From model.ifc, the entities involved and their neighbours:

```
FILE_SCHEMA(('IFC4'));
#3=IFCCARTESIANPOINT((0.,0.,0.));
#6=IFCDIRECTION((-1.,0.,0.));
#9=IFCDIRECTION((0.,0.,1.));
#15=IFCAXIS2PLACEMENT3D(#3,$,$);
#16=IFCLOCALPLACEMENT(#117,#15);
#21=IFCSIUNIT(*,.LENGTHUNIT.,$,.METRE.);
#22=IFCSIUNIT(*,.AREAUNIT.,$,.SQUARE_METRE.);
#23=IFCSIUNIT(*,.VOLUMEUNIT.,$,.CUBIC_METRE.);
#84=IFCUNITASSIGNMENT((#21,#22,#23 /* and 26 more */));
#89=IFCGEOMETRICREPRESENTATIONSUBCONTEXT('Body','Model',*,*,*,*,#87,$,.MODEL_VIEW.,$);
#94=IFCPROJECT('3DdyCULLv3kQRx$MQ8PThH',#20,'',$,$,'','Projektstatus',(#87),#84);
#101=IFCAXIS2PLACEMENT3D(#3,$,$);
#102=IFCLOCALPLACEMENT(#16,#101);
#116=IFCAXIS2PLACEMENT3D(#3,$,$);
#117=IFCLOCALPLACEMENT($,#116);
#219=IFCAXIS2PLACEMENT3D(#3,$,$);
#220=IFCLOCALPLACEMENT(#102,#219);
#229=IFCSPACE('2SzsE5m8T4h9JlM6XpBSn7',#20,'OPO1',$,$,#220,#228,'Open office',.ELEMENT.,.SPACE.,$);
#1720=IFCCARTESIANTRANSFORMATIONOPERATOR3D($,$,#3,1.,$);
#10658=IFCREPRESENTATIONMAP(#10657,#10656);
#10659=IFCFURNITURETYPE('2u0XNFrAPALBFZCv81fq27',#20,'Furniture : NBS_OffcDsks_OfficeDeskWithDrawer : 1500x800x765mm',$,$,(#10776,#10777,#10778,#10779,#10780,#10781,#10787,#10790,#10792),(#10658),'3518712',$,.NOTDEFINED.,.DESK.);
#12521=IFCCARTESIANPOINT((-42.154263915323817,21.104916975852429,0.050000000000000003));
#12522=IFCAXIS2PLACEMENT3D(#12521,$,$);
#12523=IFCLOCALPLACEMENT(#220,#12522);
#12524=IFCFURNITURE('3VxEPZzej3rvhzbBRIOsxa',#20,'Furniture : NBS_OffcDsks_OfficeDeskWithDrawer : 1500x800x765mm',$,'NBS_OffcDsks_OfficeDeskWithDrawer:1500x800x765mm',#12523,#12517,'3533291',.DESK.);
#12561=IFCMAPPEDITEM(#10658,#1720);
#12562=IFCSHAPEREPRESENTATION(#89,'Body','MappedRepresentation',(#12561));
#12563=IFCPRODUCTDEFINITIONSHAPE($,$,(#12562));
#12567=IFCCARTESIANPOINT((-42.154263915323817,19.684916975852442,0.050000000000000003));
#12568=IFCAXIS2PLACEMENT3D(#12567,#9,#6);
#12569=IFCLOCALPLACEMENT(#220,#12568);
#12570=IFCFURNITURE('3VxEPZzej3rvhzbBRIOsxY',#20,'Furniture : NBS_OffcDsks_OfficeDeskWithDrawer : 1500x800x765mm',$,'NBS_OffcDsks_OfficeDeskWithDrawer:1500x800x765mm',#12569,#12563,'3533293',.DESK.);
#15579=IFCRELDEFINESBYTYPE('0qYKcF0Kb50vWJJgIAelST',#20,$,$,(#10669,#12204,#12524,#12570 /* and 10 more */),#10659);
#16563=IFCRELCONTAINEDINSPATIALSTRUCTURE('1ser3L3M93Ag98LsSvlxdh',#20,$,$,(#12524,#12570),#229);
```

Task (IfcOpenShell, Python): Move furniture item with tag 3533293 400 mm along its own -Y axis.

```python
import ifcopenshell
import ifcopenshell.api.geometry
import ifcopenshell.util.placement
import ifcopenshell.util.unit

model = ifcopenshell.open("model.ifc")
unit_scale = ifcopenshell.util.unit.calculate_unit_scale(model)

item = model.by_guid("3VxEPZzej3rvhzbBRIOsxY")
matrix = ifcopenshell.util.placement.get_local_placement(item.ObjectPlacement)
matrix[:3, 3] -= matrix[:3, 1] * 0.4 / unit_scale
ifcopenshell.api.geometry.edit_object_placement(model, product=item, matrix=matrix, is_si=False)

print(ifcopenshell.util.placement.get_local_placement(item.ObjectPlacement).round(3) + 0.0)

model.write("model_v2.ifc")
```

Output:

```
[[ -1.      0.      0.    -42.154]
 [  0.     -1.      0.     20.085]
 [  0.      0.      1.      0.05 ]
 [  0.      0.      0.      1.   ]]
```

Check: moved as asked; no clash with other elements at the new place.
